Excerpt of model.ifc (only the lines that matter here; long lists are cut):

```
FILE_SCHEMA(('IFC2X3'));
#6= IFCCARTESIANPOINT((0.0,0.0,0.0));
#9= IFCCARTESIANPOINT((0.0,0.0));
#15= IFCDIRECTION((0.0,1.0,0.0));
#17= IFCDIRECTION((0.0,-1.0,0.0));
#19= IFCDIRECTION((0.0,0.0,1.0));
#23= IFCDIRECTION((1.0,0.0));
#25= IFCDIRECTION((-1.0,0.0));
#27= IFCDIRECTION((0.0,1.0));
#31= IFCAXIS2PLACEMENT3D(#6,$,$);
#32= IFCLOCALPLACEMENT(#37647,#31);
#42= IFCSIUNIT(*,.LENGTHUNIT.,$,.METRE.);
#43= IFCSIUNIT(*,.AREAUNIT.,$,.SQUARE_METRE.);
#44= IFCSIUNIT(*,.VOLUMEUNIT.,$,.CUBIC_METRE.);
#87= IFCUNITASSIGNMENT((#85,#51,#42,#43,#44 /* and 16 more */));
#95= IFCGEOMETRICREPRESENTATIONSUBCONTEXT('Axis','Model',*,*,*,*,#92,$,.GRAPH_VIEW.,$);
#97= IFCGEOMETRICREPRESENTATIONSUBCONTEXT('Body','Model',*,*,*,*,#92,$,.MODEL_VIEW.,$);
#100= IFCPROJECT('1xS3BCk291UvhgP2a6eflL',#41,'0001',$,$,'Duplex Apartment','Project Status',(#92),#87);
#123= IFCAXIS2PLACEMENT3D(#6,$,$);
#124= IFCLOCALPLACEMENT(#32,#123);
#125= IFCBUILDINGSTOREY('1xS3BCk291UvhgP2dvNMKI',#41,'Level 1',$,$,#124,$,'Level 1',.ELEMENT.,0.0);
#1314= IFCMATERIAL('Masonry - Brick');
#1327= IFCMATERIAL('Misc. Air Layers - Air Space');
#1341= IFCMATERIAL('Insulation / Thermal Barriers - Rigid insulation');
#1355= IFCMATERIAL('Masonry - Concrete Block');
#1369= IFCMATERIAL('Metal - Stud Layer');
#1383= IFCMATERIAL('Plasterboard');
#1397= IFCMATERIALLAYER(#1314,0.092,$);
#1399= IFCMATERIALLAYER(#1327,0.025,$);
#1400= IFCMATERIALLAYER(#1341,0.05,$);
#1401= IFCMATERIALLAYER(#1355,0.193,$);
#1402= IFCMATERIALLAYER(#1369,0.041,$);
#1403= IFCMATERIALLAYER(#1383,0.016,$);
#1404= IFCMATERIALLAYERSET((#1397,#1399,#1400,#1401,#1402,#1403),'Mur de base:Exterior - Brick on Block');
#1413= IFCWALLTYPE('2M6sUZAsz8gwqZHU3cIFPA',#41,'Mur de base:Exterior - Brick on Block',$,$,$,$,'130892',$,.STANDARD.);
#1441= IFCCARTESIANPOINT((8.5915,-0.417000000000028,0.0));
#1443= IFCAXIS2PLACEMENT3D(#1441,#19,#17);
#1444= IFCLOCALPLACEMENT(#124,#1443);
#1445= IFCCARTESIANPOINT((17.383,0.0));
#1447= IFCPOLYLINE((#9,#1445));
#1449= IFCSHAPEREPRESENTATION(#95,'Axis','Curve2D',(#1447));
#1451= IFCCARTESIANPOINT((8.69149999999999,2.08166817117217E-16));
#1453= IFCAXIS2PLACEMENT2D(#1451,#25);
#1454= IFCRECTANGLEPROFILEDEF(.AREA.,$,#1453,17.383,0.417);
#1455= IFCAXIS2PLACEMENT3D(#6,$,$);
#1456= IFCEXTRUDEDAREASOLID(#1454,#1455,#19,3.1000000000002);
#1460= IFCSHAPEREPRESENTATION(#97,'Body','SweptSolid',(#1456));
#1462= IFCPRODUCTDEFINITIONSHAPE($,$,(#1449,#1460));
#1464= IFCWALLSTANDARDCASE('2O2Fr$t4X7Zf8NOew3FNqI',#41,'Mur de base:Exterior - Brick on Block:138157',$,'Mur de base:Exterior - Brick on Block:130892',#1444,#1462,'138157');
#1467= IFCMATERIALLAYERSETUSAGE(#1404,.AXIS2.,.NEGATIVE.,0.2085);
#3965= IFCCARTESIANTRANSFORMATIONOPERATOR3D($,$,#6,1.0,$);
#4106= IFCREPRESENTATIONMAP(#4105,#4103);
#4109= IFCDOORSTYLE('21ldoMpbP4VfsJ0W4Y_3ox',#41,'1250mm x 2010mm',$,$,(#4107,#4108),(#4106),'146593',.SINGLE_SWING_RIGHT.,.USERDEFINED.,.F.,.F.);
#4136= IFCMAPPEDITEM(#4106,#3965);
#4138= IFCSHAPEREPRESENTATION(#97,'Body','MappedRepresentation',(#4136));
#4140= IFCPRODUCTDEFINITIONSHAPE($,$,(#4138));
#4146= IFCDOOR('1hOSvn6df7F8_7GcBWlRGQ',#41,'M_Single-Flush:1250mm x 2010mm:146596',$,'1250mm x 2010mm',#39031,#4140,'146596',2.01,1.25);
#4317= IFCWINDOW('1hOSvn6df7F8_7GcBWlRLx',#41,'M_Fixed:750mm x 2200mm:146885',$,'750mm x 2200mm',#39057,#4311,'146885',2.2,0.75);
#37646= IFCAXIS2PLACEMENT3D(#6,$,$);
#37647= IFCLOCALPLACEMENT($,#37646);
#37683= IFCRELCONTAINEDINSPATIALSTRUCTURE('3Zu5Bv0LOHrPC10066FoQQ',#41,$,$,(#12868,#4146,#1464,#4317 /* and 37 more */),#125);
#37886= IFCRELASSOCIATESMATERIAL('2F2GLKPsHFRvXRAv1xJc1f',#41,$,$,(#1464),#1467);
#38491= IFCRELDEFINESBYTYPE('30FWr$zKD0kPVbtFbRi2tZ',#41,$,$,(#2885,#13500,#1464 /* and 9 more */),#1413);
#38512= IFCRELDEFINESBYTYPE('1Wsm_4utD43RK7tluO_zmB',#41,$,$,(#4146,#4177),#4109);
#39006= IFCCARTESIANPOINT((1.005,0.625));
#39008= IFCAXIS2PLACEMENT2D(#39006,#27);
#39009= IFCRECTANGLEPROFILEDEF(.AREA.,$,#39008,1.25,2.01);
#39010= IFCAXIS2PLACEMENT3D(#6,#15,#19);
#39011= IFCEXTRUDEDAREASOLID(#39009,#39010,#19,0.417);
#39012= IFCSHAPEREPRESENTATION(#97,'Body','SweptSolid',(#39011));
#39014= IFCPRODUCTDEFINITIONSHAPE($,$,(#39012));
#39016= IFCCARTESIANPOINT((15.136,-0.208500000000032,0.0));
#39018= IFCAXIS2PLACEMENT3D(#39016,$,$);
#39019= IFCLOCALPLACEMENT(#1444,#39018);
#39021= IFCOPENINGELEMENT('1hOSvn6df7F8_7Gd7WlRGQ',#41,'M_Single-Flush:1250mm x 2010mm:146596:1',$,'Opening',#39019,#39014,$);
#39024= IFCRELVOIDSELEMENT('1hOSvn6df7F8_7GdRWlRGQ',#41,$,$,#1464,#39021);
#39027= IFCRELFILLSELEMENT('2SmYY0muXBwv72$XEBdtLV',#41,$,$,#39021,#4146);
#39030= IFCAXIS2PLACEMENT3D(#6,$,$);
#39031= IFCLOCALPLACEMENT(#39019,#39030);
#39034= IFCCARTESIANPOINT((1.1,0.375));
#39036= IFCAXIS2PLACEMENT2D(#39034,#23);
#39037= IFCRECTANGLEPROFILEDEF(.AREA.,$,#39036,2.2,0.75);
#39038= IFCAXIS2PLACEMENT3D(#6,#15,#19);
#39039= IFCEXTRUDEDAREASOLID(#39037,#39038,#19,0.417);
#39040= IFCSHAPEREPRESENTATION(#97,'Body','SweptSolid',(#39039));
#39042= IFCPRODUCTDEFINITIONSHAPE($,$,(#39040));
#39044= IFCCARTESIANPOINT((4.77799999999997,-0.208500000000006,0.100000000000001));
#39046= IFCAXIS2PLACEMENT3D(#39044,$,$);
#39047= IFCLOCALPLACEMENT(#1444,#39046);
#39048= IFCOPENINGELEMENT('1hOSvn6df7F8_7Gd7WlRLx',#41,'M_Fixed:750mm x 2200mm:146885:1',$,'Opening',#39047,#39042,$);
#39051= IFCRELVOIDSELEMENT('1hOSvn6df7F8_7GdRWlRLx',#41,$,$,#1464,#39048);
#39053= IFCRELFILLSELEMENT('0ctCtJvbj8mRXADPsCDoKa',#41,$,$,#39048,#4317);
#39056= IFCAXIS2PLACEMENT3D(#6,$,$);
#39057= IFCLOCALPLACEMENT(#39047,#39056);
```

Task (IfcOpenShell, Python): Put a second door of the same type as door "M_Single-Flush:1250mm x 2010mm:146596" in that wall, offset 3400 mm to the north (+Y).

```python
import ifcopenshell
import ifcopenshell.api.feature
import ifcopenshell.api.geometry
import ifcopenshell.api.root
import ifcopenshell.geom
import ifcopenshell.util.element
import ifcopenshell.util.placement
import ifcopenshell.util.shape

model = ifcopenshell.open("model.ifc")
settings = ifcopenshell.geom.settings()


def volume(element):
    """Net volume in cubic metres, openings subtracted."""
    shape = ifcopenshell.geom.create_shape(settings, element)
    return ifcopenshell.util.shape.get_volume(shape.geometry)


def reuse_history(source, copy):
    """copy_class also copies each property set's owner history, people and application; keep the originals."""
    for rel in copy.IsDefinedBy:
        if rel.is_a("IfcRelDefinesByProperties") and (history := rel.RelatingPropertyDefinition.OwnerHistory):
            rel.RelatingPropertyDefinition.OwnerHistory = source.OwnerHistory
            ifcopenshell.util.element.remove_deep2(model, history)


door = model.by_guid("1hOSvn6df7F8_7GcBWlRGQ")
opening = door.FillsVoids[0].RelatingOpeningElement
wall = opening.VoidsElements[0].RelatingBuildingElement
before = volume(wall)
shift = ifcopenshell.util.placement.get_local_placement(wall.ObjectPlacement)[:3, 0] * -3.4

# copy_class copies the void relationship, type, container and properties, but no geometry.
new_opening = ifcopenshell.api.root.copy_class(model, product=opening)
new_opening.Representation = ifcopenshell.util.element.copy_deep(
    model, opening.Representation, exclude=["IfcGeometricRepresentationContext", "IfcRepresentationMap"]
)
new_opening.Name = "M_Single-Flush:1250mm x 2010mm"
new_door = ifcopenshell.api.root.copy_class(model, product=door)
new_door.Representation = ifcopenshell.util.element.copy_deep(
    model, door.Representation, exclude=["IfcGeometricRepresentationContext", "IfcRepresentationMap"]
)
new_door.Name = "M_Single-Flush:1250mm x 2010mm"
new_door.Tag = None
reuse_history(door, new_door)
fills = ifcopenshell.api.feature.add_filling(model, opening=new_opening, element=new_door)
fills.OwnerHistory = new_door.OwnerHistory  # required in IFC2X3

for old, new in ((opening, new_opening), (door, new_door)):
    matrix = ifcopenshell.util.placement.get_local_placement(old.ObjectPlacement)
    matrix[:3, 3] += shift
    ifcopenshell.api.geometry.edit_object_placement(model, product=new, matrix=matrix, is_si=False)

after = volume(wall)

print(f"wall volume {before:.3f} -> {after:.3f} m3")

model.write("model-out.ifc")
```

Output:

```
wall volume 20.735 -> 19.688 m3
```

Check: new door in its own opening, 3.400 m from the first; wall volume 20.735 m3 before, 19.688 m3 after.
